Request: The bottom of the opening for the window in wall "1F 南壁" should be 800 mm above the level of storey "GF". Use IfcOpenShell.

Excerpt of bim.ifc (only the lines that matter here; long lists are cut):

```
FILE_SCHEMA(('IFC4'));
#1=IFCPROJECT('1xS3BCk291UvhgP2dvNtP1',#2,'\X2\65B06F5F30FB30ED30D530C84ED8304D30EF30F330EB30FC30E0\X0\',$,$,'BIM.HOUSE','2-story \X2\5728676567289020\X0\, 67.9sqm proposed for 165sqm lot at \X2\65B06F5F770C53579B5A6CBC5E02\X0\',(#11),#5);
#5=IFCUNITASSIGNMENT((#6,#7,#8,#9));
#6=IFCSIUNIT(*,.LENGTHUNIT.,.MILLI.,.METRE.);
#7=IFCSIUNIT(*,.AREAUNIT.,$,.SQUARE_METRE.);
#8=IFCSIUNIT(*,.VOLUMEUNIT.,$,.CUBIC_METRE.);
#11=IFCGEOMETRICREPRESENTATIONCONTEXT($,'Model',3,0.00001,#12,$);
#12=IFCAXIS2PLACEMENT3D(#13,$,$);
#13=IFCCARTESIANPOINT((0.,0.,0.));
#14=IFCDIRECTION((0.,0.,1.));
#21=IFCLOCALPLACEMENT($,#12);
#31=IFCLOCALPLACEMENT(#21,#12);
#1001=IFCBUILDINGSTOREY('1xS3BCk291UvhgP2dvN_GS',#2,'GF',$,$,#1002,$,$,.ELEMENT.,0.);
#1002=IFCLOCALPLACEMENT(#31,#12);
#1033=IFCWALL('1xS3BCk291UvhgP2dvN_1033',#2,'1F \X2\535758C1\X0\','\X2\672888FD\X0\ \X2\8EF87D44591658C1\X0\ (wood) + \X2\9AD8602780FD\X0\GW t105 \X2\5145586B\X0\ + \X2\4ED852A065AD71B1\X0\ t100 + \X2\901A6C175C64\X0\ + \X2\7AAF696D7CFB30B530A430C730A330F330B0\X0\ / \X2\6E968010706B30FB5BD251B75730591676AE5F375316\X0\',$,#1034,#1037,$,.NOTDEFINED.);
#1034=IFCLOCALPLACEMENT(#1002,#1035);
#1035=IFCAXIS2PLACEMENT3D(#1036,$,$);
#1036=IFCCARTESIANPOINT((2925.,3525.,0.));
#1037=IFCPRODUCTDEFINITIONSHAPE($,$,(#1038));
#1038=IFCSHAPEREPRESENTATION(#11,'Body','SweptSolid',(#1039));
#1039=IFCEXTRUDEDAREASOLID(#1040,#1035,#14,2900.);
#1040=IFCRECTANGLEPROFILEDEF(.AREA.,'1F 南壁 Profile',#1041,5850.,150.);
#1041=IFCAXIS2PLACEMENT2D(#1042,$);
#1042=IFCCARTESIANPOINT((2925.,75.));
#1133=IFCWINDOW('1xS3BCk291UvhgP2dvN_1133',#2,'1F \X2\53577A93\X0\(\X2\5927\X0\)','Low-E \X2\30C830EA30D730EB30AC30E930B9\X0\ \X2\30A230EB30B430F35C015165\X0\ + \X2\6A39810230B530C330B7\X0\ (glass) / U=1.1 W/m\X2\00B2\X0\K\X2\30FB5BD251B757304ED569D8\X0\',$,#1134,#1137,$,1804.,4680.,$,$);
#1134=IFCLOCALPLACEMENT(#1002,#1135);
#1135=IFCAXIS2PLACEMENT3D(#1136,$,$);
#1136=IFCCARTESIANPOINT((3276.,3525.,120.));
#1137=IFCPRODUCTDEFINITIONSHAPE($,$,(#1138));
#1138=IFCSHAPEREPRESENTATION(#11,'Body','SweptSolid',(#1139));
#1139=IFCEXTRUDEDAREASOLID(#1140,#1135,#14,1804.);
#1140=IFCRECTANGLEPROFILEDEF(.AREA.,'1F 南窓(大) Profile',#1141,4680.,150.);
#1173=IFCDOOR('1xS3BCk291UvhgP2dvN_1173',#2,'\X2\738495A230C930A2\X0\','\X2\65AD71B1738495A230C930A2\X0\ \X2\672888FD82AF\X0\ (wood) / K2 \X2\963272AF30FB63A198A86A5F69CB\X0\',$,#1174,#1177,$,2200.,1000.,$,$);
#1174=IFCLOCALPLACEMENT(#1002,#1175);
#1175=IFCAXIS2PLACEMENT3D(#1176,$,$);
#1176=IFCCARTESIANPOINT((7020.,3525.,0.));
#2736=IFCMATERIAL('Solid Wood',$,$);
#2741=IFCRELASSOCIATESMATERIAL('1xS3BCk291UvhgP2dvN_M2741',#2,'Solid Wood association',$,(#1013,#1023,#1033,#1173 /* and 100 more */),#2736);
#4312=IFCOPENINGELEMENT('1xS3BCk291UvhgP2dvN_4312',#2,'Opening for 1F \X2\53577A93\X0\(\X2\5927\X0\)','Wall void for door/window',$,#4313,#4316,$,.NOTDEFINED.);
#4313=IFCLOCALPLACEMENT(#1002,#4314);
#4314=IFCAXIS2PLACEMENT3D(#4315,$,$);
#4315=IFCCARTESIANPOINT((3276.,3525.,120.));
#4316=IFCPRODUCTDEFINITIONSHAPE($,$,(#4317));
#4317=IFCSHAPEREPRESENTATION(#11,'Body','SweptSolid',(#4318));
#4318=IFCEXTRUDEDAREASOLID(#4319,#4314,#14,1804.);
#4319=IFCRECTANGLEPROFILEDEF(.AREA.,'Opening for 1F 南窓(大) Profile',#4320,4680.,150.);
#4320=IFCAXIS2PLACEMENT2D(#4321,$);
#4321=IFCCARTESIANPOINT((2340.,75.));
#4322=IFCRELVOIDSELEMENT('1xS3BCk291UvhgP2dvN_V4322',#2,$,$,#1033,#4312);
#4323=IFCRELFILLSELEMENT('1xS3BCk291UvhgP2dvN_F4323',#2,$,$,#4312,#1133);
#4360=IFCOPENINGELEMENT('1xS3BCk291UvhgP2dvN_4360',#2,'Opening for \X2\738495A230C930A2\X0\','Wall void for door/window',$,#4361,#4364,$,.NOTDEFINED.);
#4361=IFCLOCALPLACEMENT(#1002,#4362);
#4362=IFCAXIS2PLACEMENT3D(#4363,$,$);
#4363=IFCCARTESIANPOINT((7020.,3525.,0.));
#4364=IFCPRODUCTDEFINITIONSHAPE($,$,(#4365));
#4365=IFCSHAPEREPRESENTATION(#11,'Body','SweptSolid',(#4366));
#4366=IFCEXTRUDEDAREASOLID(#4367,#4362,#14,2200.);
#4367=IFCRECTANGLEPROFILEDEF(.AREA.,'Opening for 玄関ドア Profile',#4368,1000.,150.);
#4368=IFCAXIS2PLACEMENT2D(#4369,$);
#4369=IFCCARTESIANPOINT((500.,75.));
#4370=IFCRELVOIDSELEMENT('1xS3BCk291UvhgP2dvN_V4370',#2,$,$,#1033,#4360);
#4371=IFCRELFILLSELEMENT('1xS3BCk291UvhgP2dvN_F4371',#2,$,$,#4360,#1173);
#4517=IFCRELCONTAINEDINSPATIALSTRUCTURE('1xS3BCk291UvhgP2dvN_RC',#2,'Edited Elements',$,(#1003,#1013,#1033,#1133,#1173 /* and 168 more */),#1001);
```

```python
import numpy as np
import ifcopenshell
import ifcopenshell.api.geometry
import ifcopenshell.geom
import ifcopenshell.util.element
import ifcopenshell.util.placement
import ifcopenshell.util.shape
import ifcopenshell.util.unit

model = ifcopenshell.open("bim.ifc")
unit_scale = ifcopenshell.util.unit.calculate_unit_scale(model)

window = model.by_guid("1xS3BCk291UvhgP2dvN_1133")
opening = window.FillsVoids[0].RelatingOpeningElement
storey = ifcopenshell.util.element.get_container(window, ifc_class="IfcBuildingStorey")
level = ifcopenshell.util.placement.get_local_placement(storey.ObjectPlacement)[2, 3]

# The opening's origin need not be at the sill, so measure its lowest point.
shape = ifcopenshell.geom.create_shape(ifcopenshell.geom.settings(), opening)
bottom = ifcopenshell.util.shape.get_shape_bottom_elevation(shape, shape.geometry) / unit_scale
dz = level + 0.8 / unit_scale - bottom

shift = np.array([0.0, 0.0, dz])
# The window is not placed relative to its opening, so move both.
for product in (opening, window):
    matrix = ifcopenshell.util.placement.get_local_placement(product.ObjectPlacement)
    matrix[:3, 3] += shift
    ifcopenshell.api.geometry.edit_object_placement(model, product=product, matrix=matrix, is_si=False)

print(f"moved by {dz * unit_scale:+.3f} m")

model.write("bim_rev.ifc")
```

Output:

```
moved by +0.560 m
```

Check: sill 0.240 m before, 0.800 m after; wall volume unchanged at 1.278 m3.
